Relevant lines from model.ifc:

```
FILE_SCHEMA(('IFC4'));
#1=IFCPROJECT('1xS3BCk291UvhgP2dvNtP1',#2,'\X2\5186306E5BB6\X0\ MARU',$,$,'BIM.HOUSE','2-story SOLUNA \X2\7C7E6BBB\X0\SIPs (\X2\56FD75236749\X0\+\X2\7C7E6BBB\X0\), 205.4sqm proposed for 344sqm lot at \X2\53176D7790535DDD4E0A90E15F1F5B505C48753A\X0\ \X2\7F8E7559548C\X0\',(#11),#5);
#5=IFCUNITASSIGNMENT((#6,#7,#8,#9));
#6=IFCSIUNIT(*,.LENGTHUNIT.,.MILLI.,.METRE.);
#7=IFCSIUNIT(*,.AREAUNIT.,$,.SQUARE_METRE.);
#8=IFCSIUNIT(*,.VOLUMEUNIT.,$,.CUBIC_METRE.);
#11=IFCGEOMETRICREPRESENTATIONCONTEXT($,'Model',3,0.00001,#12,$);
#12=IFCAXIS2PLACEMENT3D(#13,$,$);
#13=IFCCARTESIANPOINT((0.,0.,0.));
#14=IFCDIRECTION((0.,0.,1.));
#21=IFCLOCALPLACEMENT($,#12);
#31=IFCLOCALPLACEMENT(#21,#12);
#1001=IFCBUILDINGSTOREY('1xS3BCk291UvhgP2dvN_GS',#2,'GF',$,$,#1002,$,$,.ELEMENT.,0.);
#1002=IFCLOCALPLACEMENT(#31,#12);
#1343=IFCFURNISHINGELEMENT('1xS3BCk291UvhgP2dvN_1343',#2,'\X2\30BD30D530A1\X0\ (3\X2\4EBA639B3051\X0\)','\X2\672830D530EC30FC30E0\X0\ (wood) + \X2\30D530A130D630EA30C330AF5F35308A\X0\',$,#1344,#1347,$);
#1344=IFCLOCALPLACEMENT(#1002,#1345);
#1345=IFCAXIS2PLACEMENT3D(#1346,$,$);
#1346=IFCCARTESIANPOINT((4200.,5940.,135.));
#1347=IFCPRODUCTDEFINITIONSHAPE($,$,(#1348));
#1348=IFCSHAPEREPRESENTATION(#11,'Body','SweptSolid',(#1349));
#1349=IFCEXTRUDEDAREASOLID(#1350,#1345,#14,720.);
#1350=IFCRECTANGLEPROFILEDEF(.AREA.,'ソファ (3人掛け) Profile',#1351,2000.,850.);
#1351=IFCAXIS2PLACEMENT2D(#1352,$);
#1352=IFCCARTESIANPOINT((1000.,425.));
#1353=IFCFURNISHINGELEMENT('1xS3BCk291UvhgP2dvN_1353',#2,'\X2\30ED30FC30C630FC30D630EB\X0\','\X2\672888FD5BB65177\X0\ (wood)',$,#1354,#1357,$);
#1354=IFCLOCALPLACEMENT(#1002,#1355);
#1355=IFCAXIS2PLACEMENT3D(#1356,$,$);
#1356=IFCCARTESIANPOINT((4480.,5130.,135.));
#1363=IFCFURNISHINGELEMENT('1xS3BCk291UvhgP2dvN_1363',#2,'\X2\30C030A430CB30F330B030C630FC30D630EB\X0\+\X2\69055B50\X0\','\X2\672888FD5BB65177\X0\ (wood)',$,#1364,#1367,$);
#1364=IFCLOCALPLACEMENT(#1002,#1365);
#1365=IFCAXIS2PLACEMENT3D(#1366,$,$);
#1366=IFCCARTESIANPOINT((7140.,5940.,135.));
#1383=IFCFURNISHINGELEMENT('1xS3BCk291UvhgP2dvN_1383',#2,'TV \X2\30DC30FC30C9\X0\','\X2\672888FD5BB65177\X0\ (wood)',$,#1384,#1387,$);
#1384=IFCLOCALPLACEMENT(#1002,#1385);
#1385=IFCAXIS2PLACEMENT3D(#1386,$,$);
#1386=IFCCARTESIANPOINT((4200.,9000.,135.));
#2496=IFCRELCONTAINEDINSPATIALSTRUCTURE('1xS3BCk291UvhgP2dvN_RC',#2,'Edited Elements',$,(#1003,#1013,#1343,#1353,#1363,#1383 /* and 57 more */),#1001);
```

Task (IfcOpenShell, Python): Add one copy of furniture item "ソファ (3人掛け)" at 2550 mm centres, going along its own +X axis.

```python
import ifcopenshell
import ifcopenshell.api.geometry
import ifcopenshell.api.root
import ifcopenshell.util.element
import ifcopenshell.util.placement
import ifcopenshell.util.unit

model = ifcopenshell.open("model.ifc")
unit_scale = ifcopenshell.util.unit.calculate_unit_scale(model)


def reuse_history(source, copy):
    """copy_class also copies each property set's owner history, people and application; keep the originals."""
    for rel in copy.IsDefinedBy:
        if rel.is_a("IfcRelDefinesByProperties") and (history := rel.RelatingPropertyDefinition.OwnerHistory):
            rel.RelatingPropertyDefinition.OwnerHistory = source.OwnerHistory
            ifcopenshell.util.element.remove_deep2(model, history)


source = model.by_guid("1xS3BCk291UvhgP2dvN_1343")
base = ifcopenshell.util.placement.get_local_placement(source.ObjectPlacement)
step = base[:3, 0] * 2.55 / unit_scale

for i in range(1, 2):
    copy = ifcopenshell.api.root.copy_class(model, product=source)
    copy.Representation = ifcopenshell.util.element.copy_deep(
        model, source.Representation, exclude=["IfcGeometricRepresentationContext", "IfcRepresentationMap"]
    )
    reuse_history(source, copy)
    matrix = base.copy()
    matrix[:3, 3] += i * step
    print("added at", matrix[:3, 3].round(3) + 0.0)
    ifcopenshell.api.geometry.edit_object_placement(model, product=copy, matrix=matrix, is_si=False)

model.write("model-out.ifc")
```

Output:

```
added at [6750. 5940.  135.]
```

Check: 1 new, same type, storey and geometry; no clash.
